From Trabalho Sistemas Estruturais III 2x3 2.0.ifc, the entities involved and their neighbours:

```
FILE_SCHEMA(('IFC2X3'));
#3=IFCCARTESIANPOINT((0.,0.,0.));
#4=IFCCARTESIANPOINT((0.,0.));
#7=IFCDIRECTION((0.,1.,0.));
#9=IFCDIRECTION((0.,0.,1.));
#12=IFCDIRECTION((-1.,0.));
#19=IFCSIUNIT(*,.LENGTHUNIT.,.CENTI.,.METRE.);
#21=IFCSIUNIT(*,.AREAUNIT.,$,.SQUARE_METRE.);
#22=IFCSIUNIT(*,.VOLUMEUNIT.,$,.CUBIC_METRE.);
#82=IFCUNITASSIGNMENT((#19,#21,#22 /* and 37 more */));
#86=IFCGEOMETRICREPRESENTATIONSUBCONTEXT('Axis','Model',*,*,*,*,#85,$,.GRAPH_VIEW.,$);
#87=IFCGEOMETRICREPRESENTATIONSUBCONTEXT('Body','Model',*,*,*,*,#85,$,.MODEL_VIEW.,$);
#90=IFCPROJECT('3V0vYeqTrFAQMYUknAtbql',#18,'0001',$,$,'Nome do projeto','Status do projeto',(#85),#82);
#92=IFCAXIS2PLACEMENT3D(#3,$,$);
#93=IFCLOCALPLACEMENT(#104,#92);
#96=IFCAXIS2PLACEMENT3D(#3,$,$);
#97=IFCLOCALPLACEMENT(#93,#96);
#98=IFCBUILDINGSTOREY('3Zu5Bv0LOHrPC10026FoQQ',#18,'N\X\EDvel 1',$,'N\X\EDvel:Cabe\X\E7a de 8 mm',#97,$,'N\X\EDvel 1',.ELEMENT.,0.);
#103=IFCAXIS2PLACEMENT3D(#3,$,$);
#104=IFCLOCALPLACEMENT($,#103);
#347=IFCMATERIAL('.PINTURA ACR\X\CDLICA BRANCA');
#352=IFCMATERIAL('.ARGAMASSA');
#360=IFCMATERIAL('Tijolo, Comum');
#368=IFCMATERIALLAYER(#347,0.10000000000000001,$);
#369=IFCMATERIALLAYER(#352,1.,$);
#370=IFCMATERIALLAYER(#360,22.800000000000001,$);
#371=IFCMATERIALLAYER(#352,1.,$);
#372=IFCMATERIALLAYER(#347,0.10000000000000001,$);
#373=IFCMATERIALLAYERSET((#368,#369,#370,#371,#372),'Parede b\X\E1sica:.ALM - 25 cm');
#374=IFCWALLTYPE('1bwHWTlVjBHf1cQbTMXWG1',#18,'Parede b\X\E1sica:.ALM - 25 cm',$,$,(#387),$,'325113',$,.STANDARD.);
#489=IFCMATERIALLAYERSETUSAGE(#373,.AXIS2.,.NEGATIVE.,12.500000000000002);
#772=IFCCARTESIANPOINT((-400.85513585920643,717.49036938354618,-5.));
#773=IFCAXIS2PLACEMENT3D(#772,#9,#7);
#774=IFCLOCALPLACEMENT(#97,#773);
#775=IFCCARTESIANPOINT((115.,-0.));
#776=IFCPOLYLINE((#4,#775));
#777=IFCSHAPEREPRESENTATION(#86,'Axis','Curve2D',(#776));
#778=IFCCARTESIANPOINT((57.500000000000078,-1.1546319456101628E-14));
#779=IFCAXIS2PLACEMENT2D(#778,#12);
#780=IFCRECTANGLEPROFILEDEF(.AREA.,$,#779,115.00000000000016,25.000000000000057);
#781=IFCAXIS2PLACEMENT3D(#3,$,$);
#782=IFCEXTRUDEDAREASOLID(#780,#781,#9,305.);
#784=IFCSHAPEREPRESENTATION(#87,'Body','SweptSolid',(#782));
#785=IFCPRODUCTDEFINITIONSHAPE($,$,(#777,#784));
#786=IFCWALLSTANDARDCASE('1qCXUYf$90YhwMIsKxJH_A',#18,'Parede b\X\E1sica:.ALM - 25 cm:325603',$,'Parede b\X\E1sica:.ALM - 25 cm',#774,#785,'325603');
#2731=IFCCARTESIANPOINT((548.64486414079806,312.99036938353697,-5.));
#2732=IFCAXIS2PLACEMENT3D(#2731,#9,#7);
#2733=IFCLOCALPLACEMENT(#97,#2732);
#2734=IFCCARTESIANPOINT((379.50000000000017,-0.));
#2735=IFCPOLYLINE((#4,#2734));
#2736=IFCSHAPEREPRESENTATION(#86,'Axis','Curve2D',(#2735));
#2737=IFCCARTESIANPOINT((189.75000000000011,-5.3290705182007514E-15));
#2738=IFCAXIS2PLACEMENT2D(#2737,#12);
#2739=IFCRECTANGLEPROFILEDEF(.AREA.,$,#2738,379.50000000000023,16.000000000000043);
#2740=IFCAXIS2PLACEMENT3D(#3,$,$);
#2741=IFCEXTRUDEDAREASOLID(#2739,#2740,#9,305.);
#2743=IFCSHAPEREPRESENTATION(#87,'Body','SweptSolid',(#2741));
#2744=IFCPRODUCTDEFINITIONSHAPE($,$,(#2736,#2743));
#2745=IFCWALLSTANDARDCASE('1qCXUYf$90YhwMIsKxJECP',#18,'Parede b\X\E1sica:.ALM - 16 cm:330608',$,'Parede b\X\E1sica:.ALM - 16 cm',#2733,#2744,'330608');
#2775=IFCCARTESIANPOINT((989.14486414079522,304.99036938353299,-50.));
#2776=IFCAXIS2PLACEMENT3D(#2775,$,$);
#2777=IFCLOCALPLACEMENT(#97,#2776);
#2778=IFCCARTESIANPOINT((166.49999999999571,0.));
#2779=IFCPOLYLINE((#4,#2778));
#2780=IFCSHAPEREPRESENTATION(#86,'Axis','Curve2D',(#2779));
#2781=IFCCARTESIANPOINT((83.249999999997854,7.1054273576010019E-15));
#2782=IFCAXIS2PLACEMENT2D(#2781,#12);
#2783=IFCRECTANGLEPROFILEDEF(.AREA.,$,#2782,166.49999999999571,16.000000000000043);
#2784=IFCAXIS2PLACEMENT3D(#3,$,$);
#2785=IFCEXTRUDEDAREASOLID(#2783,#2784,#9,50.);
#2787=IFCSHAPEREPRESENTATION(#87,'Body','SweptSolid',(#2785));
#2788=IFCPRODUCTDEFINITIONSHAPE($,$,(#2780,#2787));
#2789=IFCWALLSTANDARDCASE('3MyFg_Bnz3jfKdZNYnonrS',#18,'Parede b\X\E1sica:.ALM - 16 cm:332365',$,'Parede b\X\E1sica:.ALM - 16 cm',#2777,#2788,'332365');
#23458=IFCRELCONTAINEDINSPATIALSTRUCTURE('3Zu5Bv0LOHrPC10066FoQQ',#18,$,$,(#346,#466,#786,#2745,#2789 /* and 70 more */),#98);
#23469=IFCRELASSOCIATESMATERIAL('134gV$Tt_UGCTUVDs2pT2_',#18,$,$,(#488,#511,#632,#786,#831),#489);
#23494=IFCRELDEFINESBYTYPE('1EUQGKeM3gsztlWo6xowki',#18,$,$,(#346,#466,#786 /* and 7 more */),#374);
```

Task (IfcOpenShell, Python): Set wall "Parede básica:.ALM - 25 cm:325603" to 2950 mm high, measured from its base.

```python
import ifcopenshell
import ifcopenshell.geom
import ifcopenshell.util.representation
import ifcopenshell.util.shape
import ifcopenshell.util.unit

model = ifcopenshell.open("Trabalho Sistemas Estruturais III 2x3 2.0.ifc")
unit_scale = ifcopenshell.util.unit.calculate_unit_scale(model)
settings = ifcopenshell.geom.settings()


def volume(element):
    """Net volume in cubic metres, openings subtracted."""
    shape = ifcopenshell.geom.create_shape(settings, element)
    return ifcopenshell.util.shape.get_volume(shape.geometry)


wall = model.by_guid("1qCXUYf$90YhwMIsKxJH_A")
before = volume(wall)

body = ifcopenshell.util.representation.get_representation(wall, "Model", "Body")
solid = body.Items[0]
old_height = solid.Depth
solid.Depth = 2.95 / unit_scale
after = volume(wall)

print(f"height {old_height:g} -> {solid.Depth:g}, volume {before:.3f} -> {after:.3f} m3")

model.write("Trabalho Sistemas Estruturais III 2x3 2.0_v2.ifc")
```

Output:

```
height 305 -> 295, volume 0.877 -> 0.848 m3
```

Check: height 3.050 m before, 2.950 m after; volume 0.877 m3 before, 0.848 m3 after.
